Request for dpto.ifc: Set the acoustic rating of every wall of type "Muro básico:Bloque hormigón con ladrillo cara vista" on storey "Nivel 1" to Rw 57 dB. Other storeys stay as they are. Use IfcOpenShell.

First a look at what the model holds.

```python
import ifcopenshell
import ifcopenshell.util.element

model = ifcopenshell.open("dpto.ifc")
print(model.schema)
storey = next(s for s in model.by_type("IfcBuildingStorey") if s.Name == "Nivel 1")
walls = [e for e in ifcopenshell.util.element.get_decomposition(storey) if e.is_a("IfcWall")]
seen = {}
for e in walls:
    element_type = ifcopenshell.util.element.get_type(e)
    key = (element_type.Name if element_type != e and element_type else None, ifcopenshell.util.element.get_pset(e, "Pset_WallCommon", "AcousticRating"))
    seen[key] = seen.get(key, 0) + 1
for (name, value), count in sorted(seen.items(), key=str):
    print(count, "x", name, "|", value)
```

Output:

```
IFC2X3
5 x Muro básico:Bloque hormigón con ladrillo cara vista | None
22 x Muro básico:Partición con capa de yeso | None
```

```python
import ifcopenshell
import ifcopenshell.api.pset
import ifcopenshell.util.element

model = ifcopenshell.open("dpto.ifc")

storey = next(s for s in model.by_type("IfcBuildingStorey") if s.Name == "Nivel 1")
walls = [e for e in ifcopenshell.util.element.get_decomposition(storey) if e.is_a("IfcWall")]

count = 0
for e in walls:
    element_type = ifcopenshell.util.element.get_type(e)
    if element_type in (None, e) or element_type.Name != "Muro básico:Bloque hormigón con ladrillo cara vista":
        continue
    # add_pset returns the element's existing set when there is one.
    pset = ifcopenshell.api.pset.add_pset(model, product=e, name="Pset_WallCommon")
    ifcopenshell.api.pset.edit_pset(model, pset=pset, properties={"AcousticRating": "Rw 57 dB"})
    count += 1

print(count, "walls updated")

model.write("dpto_edited.ifc")
```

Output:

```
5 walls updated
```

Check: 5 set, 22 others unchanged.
